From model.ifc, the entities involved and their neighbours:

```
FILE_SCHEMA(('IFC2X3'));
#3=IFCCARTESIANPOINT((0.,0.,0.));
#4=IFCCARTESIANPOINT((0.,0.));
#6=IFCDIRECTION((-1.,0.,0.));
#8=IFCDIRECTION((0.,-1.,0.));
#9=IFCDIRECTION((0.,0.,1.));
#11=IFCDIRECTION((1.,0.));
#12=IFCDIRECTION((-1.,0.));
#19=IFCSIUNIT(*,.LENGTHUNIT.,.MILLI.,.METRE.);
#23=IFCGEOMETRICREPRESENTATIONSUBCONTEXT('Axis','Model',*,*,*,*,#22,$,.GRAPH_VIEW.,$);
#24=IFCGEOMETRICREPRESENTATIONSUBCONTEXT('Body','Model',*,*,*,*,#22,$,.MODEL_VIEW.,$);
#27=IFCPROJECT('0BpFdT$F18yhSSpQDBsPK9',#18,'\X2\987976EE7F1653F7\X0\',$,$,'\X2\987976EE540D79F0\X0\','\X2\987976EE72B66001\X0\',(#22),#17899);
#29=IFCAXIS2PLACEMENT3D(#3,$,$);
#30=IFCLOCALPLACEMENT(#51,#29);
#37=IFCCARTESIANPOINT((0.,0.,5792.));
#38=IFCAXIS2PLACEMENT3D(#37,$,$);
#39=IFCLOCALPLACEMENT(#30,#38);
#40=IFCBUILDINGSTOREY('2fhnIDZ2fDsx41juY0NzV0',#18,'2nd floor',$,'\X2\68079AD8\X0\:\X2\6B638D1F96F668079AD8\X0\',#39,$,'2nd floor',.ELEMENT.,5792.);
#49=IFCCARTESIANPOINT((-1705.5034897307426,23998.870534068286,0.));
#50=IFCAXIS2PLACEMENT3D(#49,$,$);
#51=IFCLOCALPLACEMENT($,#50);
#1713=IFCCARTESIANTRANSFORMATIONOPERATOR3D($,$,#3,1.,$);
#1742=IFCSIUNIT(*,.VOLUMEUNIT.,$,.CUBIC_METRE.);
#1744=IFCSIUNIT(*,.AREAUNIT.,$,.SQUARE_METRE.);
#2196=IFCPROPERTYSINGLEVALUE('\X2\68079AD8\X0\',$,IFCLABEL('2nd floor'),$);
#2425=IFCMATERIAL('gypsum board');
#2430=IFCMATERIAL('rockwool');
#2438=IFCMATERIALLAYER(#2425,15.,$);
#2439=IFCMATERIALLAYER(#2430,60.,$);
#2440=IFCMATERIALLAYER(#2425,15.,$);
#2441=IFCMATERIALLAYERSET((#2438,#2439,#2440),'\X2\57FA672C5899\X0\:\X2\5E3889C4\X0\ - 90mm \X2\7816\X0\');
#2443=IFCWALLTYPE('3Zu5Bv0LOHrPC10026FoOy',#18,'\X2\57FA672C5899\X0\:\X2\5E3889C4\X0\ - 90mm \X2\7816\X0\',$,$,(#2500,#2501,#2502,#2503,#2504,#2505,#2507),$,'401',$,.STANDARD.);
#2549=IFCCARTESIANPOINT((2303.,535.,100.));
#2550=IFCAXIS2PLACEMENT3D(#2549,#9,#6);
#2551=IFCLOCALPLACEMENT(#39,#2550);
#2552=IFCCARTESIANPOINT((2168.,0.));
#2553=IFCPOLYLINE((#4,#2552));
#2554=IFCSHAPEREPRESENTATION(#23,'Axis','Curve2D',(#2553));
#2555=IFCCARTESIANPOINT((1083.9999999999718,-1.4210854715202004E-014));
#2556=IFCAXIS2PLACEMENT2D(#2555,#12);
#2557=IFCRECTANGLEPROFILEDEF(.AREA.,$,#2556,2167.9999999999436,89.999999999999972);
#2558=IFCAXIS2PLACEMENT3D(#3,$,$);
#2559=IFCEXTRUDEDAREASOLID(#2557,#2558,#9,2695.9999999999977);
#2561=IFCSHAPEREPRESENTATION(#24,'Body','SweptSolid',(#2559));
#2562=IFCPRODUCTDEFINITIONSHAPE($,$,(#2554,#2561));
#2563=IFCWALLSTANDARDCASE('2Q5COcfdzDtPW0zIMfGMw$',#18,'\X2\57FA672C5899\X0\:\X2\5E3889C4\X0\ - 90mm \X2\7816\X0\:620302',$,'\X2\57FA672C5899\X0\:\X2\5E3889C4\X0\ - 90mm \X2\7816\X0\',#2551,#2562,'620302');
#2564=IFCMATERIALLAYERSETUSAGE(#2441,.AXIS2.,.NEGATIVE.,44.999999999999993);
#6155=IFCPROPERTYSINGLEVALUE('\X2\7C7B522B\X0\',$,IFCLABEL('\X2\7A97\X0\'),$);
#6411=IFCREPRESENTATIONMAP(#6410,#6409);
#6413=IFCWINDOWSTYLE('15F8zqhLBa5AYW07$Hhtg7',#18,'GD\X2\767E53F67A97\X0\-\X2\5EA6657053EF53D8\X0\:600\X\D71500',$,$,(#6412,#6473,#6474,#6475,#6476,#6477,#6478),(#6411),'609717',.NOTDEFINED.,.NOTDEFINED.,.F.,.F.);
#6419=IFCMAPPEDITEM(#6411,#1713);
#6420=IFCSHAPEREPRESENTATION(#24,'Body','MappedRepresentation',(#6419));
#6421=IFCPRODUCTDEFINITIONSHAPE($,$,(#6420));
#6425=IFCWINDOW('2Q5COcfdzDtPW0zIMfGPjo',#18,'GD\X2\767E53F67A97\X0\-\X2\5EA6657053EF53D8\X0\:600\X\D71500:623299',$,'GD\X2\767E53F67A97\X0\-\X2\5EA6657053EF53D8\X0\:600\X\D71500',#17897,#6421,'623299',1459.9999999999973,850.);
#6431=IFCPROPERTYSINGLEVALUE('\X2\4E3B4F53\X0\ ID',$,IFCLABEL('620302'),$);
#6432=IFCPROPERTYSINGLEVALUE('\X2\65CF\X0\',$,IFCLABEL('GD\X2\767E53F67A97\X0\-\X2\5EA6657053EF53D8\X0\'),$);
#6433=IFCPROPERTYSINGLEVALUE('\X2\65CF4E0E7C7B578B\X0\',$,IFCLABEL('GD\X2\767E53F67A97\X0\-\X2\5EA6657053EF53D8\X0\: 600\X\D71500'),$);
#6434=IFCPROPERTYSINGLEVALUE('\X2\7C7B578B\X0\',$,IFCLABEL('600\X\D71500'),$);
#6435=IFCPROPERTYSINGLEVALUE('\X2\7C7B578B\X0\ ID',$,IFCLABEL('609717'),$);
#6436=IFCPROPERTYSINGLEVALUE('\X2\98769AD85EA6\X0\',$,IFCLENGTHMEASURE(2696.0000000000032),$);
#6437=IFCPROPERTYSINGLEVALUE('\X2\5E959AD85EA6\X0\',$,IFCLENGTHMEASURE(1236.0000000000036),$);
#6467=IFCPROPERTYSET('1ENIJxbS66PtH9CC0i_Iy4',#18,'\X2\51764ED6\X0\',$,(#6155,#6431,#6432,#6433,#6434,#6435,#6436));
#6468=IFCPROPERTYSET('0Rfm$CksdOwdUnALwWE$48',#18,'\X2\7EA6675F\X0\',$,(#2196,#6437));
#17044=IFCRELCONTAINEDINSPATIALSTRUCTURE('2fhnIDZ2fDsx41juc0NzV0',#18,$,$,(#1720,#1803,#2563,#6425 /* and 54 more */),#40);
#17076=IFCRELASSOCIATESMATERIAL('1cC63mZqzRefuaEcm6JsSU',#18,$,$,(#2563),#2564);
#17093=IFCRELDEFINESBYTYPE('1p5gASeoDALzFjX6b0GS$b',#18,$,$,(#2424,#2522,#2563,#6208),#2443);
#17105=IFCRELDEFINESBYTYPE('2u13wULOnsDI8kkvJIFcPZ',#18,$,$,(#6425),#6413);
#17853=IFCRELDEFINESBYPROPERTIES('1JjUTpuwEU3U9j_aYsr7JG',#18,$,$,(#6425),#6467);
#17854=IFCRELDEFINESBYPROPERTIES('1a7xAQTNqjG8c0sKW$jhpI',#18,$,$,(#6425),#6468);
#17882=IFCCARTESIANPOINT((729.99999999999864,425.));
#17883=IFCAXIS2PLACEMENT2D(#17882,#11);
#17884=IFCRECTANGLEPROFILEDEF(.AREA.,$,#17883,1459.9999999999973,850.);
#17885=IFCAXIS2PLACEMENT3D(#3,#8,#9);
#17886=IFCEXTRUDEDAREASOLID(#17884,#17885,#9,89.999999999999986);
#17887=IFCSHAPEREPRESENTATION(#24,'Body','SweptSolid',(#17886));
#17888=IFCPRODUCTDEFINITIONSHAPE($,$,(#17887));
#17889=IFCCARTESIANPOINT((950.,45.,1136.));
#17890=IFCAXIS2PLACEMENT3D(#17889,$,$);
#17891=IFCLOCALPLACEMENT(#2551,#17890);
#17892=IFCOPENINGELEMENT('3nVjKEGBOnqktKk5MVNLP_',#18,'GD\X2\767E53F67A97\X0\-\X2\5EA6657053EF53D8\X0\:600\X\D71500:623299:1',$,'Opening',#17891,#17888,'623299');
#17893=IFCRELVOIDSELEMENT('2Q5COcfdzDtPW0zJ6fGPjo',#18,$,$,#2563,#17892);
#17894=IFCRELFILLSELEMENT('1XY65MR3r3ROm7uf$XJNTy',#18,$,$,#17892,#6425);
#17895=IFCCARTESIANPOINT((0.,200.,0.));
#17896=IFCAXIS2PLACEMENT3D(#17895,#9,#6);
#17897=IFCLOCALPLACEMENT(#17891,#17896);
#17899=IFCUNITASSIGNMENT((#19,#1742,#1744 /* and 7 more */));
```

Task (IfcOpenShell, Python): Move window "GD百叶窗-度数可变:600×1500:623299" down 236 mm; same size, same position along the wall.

```python
import numpy as np
import ifcopenshell
import ifcopenshell.api.geometry
import ifcopenshell.api.pset
import ifcopenshell.util.element
import ifcopenshell.util.placement
import ifcopenshell.util.unit

model = ifcopenshell.open("model.ifc")
unit_scale = ifcopenshell.util.unit.calculate_unit_scale(model)

window = model.by_guid("2Q5COcfdzDtPW0zIMfGPjo")
opening = window.FillsVoids[0].RelatingOpeningElement
dz = -0.236 / unit_scale

shift = np.array([0.0, 0.0, dz])
# The window is placed relative to its opening, so it follows when the opening moves.
matrix = ifcopenshell.util.placement.get_local_placement(opening.ObjectPlacement)
matrix[:3, 3] += shift
ifcopenshell.api.geometry.edit_object_placement(
    model, product=opening, matrix=matrix, is_si=False, should_transform_children=True
)

# Keep the stored heights in step.
pset = model.by_id(ifcopenshell.util.element.get_pset(window, "其他", should_inherit=False)["id"])
ifcopenshell.api.pset.edit_pset(model, pset=pset, properties={
    "顶高度": model.create_entity("IfcLengthMeasure", ifcopenshell.util.element.get_pset(window, "其他", "顶高度") + dz),
})
pset = model.by_id(ifcopenshell.util.element.get_pset(window, "约束", should_inherit=False)["id"])
ifcopenshell.api.pset.edit_pset(model, pset=pset, properties={
    "底高度": model.create_entity("IfcLengthMeasure", ifcopenshell.util.element.get_pset(window, "约束", "底高度") + dz),
})

print(f"moved by {dz * unit_scale:+.3f} m")

model.write("model_updated.ifc")
```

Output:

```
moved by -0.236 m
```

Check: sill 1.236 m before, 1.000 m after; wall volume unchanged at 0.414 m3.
